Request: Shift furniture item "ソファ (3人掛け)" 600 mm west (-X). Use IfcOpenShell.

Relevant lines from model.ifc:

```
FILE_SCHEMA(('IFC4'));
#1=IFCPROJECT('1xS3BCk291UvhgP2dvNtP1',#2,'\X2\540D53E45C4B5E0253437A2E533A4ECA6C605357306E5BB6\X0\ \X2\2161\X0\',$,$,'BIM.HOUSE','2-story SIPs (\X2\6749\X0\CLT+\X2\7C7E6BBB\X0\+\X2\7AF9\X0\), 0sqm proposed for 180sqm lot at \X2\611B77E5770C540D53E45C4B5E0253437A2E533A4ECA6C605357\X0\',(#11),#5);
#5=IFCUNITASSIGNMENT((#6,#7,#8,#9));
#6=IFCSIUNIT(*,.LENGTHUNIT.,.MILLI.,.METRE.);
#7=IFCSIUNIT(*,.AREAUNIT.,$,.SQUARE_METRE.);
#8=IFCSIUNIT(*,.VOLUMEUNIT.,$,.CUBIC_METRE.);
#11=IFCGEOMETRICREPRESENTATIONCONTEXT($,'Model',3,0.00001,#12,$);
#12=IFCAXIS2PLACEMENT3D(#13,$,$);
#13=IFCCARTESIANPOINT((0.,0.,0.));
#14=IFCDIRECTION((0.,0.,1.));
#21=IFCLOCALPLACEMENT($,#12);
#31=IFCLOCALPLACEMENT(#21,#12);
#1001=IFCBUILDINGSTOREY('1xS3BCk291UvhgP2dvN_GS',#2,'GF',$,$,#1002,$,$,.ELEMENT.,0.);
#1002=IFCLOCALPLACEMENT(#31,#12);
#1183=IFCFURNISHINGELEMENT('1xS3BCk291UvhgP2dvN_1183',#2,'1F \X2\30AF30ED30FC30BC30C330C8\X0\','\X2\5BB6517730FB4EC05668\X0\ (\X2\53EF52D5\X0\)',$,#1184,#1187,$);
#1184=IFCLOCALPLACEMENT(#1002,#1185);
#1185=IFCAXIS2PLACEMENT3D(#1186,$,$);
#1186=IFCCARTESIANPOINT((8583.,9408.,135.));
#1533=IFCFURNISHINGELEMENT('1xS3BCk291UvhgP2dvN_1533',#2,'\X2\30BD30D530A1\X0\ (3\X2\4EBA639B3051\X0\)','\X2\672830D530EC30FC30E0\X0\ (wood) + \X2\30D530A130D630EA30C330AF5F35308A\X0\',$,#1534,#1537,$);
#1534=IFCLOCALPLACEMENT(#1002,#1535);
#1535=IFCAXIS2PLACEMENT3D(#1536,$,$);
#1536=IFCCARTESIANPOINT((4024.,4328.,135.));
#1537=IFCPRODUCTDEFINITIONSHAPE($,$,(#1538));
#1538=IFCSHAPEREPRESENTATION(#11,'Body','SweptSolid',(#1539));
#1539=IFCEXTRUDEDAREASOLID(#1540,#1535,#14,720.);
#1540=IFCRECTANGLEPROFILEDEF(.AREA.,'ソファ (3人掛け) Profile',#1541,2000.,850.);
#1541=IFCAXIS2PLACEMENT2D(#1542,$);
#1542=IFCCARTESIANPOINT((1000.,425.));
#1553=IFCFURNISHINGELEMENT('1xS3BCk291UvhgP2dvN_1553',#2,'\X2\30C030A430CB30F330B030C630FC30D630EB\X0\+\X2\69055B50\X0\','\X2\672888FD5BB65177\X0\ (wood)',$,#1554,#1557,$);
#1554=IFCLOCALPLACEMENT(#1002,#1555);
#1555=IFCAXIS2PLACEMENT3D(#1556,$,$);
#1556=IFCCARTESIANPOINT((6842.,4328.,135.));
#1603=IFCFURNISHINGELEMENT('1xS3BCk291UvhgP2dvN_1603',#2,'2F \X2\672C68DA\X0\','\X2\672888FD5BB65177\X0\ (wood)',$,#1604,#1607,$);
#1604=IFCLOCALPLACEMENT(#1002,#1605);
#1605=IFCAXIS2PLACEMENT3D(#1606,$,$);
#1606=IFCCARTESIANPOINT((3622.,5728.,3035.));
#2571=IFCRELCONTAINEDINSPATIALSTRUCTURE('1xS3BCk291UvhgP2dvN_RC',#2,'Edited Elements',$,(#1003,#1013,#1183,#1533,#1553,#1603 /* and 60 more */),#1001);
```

```python
import ifcopenshell
import ifcopenshell.api.geometry
import ifcopenshell.util.placement
import ifcopenshell.util.unit

model = ifcopenshell.open("model.ifc")
unit_scale = ifcopenshell.util.unit.calculate_unit_scale(model)

item = model.by_guid("1xS3BCk291UvhgP2dvN_1533")
matrix = ifcopenshell.util.placement.get_local_placement(item.ObjectPlacement)
matrix[0, 3] -= 0.6 / unit_scale
ifcopenshell.api.geometry.edit_object_placement(model, product=item, matrix=matrix, is_si=False)

print(ifcopenshell.util.placement.get_local_placement(item.ObjectPlacement).round(3) + 0.0)

model.write("model_rev.ifc")
```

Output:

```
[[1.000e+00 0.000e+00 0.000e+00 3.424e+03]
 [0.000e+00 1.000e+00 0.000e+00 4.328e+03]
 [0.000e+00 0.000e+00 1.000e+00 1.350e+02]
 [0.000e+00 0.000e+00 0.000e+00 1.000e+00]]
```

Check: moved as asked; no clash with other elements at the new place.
